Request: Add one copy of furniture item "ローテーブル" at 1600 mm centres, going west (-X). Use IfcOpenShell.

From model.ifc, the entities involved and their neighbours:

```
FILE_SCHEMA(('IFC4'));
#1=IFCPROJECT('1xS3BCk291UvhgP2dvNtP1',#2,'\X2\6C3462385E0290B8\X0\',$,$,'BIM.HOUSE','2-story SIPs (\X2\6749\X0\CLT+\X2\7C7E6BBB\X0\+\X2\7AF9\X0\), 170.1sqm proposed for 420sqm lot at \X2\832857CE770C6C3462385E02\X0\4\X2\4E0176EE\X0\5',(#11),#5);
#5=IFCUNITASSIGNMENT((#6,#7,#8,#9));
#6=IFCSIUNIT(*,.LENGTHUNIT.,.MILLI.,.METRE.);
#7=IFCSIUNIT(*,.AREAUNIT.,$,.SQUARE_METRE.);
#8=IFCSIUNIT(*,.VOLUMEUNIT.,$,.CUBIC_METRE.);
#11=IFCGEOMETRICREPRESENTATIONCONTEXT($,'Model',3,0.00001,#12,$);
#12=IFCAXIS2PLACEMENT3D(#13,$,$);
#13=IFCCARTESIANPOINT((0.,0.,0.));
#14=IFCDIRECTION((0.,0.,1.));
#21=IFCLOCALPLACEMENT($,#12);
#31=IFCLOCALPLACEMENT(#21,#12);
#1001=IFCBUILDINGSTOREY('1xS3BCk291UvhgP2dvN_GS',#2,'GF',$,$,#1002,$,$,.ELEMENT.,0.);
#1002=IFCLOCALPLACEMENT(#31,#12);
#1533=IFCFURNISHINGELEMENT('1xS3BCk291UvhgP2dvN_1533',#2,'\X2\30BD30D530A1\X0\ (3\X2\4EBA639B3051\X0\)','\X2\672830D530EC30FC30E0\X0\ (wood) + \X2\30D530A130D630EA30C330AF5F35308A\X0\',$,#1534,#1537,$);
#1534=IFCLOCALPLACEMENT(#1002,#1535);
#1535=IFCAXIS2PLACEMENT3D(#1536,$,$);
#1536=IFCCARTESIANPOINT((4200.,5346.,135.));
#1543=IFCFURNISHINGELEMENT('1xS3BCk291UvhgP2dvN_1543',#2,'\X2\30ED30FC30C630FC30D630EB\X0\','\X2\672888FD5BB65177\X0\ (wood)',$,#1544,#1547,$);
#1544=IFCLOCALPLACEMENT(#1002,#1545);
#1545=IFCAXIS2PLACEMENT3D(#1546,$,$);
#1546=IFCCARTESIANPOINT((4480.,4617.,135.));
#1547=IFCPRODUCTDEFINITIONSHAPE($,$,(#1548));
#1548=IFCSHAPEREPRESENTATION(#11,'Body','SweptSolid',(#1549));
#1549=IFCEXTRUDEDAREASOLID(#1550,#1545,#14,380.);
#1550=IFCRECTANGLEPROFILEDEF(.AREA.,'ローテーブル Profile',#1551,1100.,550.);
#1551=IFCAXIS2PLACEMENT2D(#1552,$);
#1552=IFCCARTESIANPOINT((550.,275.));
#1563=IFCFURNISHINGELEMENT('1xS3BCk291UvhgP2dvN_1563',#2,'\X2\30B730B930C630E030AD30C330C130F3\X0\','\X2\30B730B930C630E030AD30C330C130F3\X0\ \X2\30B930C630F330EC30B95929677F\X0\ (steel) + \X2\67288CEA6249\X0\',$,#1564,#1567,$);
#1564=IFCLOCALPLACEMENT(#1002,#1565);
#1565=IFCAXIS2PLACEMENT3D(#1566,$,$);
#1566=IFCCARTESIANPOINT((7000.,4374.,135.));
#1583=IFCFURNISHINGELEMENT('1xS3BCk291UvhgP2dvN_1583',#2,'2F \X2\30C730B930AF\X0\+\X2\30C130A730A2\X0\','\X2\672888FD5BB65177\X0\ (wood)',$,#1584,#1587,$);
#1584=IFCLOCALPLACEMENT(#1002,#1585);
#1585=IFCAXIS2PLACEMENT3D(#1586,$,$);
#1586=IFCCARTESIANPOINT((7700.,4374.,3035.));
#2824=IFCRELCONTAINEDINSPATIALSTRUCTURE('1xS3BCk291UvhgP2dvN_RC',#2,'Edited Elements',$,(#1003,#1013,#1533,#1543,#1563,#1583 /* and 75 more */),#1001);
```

```python
import numpy as np
import ifcopenshell
import ifcopenshell.api.geometry
import ifcopenshell.api.root
import ifcopenshell.util.element
import ifcopenshell.util.placement
import ifcopenshell.util.unit

model = ifcopenshell.open("model.ifc")
unit_scale = ifcopenshell.util.unit.calculate_unit_scale(model)


def reuse_history(source, copy):
    """copy_class also copies each property set's owner history, people and application; keep the originals."""
    for rel in copy.IsDefinedBy:
        if rel.is_a("IfcRelDefinesByProperties") and (history := rel.RelatingPropertyDefinition.OwnerHistory):
            rel.RelatingPropertyDefinition.OwnerHistory = source.OwnerHistory
            ifcopenshell.util.element.remove_deep2(model, history)


source = model.by_id(1543)
base = ifcopenshell.util.placement.get_local_placement(source.ObjectPlacement)
step = np.array([-1.0, 0.0, 0.0]) * 1.6 / unit_scale

for i in range(1, 2):
    copy = ifcopenshell.api.root.copy_class(model, product=source)
    copy.Representation = ifcopenshell.util.element.copy_deep(
        model, source.Representation, exclude=["IfcGeometricRepresentationContext", "IfcRepresentationMap"]
    )
    reuse_history(source, copy)
    matrix = base.copy()
    matrix[:3, 3] += i * step
    print("added at", matrix[:3, 3].round(3) + 0.0)
    ifcopenshell.api.geometry.edit_object_placement(model, product=copy, matrix=matrix, is_si=False)

model.write("model_updated.ifc")
```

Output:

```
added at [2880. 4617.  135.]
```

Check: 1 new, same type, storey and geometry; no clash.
